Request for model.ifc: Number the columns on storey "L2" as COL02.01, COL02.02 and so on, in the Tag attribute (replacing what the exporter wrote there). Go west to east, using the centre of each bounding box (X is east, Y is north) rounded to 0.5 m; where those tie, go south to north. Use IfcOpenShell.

First a look at what the model holds.

```python
import ifcopenshell
import ifcopenshell.util.element
import ifcopenshell.util.placement

model = ifcopenshell.open("model.ifc")
print(model.schema)
storey = next(s for s in model.by_type("IfcBuildingStorey") if s.Name == "L2")
columns = [e for e in ifcopenshell.util.element.get_decomposition(storey) if e.is_a("IfcColumn")]
for e in sorted(columns, key=lambda e: e.id()):
    origin = ifcopenshell.util.placement.get_local_placement(e.ObjectPlacement)[:3, 3]
    print(e.id(), e.Tag, e.Name, origin.round(2) + 0.0, sep=" | ")
```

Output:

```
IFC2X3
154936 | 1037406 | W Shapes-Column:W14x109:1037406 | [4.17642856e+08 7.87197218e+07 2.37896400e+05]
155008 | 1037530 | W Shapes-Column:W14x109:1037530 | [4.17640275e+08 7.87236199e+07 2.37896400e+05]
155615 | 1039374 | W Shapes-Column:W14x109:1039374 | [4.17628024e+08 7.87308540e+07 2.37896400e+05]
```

```python
import ifcopenshell
import ifcopenshell.geom
import ifcopenshell.util.element
import ifcopenshell.util.shape

model = ifcopenshell.open("model.ifc")
settings = ifcopenshell.geom.settings()
settings.set("use-world-coords", True)


def centre(element):
    shape = ifcopenshell.geom.create_shape(settings, element)
    return ifcopenshell.util.shape.get_bbox_centroid(shape.geometry)


storey = next(s for s in model.by_type("IfcBuildingStorey") if s.Name == "L2")
columns = [e for e in ifcopenshell.util.element.get_decomposition(storey) if e.is_a("IfcColumn")]

# Insertion points can sit at a corner or the storey origin, so sort by the geometry (in metres).
centres = {e: centre(e) for e in columns}
columns.sort(key=lambda e: (round(centres[e][0] / 0.5), centres[e][1]))

for i, e in enumerate(columns, start=1):
    number = f"COL02.{i:02d}"
    e.Tag = number
    print(e.id(), number)

model.write("model_updated.ifc")
```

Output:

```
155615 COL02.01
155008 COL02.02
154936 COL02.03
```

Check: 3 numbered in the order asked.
